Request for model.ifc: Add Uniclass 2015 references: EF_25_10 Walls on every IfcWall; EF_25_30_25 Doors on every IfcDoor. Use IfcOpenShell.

First a look at what the model holds.

```python
import ifcopenshell

model = ifcopenshell.open("model.ifc")
print(model.schema)
print("classifications:", [c.Name for c in model.by_type("IfcClassification")])
for ifc_class in ("IfcDoor", "IfcRoof", "IfcStair", "IfcWall", "IfcWindow"):
    print(ifc_class, len(model.by_type(ifc_class)))
```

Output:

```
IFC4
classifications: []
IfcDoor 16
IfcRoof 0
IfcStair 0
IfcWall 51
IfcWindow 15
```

```python
import ifcopenshell
import ifcopenshell.api.classification

model = ifcopenshell.open("model.ifc")

system = ifcopenshell.api.classification.add_classification(model, classification="Uniclass 2015")

codes = {
    "IfcWall": ("EF_25_10", "Walls"),
    "IfcDoor": ("EF_25_30_25", "Doors"),
}
for ifc_class, (code, name) in codes.items():
    products = model.by_type(ifc_class)
    ifcopenshell.api.classification.add_reference(
        model, products=products, classification=system, identification=code, name=name
    )
    print(code, len(products))

model.write("model_edited.ifc")
```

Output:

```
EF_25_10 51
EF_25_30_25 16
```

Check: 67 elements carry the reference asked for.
